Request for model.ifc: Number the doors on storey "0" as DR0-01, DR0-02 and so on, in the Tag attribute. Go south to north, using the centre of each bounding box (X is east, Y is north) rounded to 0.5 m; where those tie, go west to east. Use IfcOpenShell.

First a look at what the model holds.

```python
import ifcopenshell
import ifcopenshell.util.element
import ifcopenshell.util.placement

model = ifcopenshell.open("model.ifc")
print(model.schema)
storey = next(s for s in model.by_type("IfcBuildingStorey") if s.Name == "0")
doors = [e for e in ifcopenshell.util.element.get_decomposition(storey) if e.is_a("IfcDoor")]
for e in sorted(doors, key=lambda e: e.id()):
    origin = ifcopenshell.util.placement.get_local_placement(e.ObjectPlacement)[:3, 3]
    print(e.id(), e.Tag, e.Name, origin.round(2) + 0.0, sep=" | ")
```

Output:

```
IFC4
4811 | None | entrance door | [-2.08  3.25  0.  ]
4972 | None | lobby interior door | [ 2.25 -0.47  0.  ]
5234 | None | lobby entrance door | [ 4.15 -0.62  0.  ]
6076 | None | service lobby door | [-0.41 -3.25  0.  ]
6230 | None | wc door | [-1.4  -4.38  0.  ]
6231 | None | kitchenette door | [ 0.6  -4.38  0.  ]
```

```python
import ifcopenshell
import ifcopenshell.geom
import ifcopenshell.util.element
import ifcopenshell.util.shape

model = ifcopenshell.open("model.ifc")
settings = ifcopenshell.geom.settings()
settings.set("use-world-coords", True)


def centre(element):
    shape = ifcopenshell.geom.create_shape(settings, element)
    return ifcopenshell.util.shape.get_bbox_centroid(shape.geometry)


storey = next(s for s in model.by_type("IfcBuildingStorey") if s.Name == "0")
doors = [e for e in ifcopenshell.util.element.get_decomposition(storey) if e.is_a("IfcDoor")]

# Insertion points can sit at a corner or the storey origin, so sort by the geometry (in metres).
centres = {e: centre(e) for e in doors}
doors.sort(key=lambda e: (round(centres[e][1] / 0.5), centres[e][0]))

for i, e in enumerate(doors, start=1):
    number = f"DR0-{i:02d}"
    e.Tag = number
    print(e.id(), number)

model.write("model_edited.ifc")
```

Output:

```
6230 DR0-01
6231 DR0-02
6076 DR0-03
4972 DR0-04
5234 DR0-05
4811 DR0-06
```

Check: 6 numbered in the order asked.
